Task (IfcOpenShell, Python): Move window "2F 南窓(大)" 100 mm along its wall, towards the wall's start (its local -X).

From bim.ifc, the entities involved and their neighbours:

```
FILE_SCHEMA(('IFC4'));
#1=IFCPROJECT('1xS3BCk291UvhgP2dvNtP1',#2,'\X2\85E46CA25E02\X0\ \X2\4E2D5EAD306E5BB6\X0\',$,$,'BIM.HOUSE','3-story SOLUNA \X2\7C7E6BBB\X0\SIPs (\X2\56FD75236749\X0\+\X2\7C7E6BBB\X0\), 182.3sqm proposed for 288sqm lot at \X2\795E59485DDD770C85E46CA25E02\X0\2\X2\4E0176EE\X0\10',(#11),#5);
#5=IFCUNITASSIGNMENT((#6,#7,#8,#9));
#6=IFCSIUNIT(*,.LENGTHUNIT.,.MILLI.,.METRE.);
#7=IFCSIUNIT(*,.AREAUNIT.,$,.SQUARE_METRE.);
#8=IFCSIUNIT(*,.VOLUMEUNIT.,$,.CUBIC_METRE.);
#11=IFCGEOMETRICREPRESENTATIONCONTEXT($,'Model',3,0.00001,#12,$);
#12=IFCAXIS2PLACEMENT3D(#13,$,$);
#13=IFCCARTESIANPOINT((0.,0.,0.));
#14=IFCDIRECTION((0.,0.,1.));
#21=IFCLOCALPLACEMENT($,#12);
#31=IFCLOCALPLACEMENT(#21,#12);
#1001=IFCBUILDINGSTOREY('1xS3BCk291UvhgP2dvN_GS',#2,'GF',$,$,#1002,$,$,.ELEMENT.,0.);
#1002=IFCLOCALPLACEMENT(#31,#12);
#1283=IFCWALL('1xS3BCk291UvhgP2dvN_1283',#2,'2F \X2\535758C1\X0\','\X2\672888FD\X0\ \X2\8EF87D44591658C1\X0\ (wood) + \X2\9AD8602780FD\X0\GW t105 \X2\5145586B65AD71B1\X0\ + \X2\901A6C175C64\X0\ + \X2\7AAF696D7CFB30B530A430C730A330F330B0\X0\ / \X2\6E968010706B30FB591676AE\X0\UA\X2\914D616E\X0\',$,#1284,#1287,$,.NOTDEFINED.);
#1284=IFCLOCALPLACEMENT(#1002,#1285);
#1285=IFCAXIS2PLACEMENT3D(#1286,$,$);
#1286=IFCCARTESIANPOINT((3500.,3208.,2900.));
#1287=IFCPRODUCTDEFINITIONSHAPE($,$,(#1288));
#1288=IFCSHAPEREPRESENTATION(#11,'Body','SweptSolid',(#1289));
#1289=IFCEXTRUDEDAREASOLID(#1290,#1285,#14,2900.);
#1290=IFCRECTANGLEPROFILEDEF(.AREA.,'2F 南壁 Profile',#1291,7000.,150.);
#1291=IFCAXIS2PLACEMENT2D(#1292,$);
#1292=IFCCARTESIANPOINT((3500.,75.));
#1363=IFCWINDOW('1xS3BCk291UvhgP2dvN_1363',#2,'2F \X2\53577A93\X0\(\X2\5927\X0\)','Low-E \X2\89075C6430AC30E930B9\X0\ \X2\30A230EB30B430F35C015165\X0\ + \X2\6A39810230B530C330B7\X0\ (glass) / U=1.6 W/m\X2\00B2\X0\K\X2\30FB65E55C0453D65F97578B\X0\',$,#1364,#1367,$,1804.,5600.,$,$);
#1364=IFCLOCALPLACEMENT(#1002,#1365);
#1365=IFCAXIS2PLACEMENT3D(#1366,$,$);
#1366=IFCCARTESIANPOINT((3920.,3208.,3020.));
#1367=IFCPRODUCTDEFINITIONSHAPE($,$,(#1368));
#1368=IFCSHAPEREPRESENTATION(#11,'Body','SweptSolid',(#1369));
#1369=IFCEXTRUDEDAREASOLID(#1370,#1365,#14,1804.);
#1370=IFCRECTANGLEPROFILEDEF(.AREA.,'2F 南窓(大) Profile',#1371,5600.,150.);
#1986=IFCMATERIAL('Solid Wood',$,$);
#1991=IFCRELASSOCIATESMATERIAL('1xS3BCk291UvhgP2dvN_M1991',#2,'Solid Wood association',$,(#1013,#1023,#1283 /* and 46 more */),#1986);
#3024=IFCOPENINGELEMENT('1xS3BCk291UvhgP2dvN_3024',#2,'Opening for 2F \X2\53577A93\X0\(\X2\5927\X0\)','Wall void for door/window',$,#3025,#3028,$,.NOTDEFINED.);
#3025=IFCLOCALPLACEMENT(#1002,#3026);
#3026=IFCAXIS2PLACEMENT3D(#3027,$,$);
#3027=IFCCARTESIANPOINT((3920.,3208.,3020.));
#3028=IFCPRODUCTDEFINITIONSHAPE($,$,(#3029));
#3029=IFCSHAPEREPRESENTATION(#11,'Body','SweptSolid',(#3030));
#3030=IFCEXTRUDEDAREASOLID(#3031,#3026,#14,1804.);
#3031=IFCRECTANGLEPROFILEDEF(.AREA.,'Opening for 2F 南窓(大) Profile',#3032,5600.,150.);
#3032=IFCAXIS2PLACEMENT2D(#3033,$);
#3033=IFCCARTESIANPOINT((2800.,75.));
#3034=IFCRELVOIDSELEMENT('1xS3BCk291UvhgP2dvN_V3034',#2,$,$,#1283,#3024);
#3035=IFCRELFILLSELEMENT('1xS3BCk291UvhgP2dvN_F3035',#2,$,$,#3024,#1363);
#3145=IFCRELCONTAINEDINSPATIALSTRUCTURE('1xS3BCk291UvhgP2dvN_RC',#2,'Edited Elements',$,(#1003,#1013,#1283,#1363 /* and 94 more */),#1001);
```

```python
import ifcopenshell
import ifcopenshell.api.geometry
import ifcopenshell.util.placement

model = ifcopenshell.open("bim.ifc")

window = model.by_guid("1xS3BCk291UvhgP2dvN_1363")
opening = window.FillsVoids[0].RelatingOpeningElement
wall = opening.VoidsElements[0].RelatingBuildingElement

wall_matrix = ifcopenshell.util.placement.get_local_placement(wall.ObjectPlacement)
shift = wall_matrix[:3, 0] * -100.0
before = ifcopenshell.util.placement.get_local_placement(window.ObjectPlacement)[:3, 3].copy()

# The window is not placed relative to its opening, so move both.
for product in (opening, window):
    matrix = ifcopenshell.util.placement.get_local_placement(product.ObjectPlacement)
    matrix[:3, 3] += shift
    ifcopenshell.api.geometry.edit_object_placement(model, product=product, matrix=matrix, is_si=False)

after = ifcopenshell.util.placement.get_local_placement(window.ObjectPlacement)[:3, 3]
print("window moved by", (after - before).round(3) + 0.0)

model.write("bim_v2.ifc")
```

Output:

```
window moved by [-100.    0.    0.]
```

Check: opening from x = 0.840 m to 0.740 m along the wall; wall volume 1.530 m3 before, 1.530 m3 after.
